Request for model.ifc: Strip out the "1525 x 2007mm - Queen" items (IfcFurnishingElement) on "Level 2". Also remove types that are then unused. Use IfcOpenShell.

First a look at what the model holds.

```python
import ifcopenshell
import ifcopenshell.util.element

model = ifcopenshell.open("model.ifc")
print(model.schema)
storey = next(s for s in model.by_type("IfcBuildingStorey") if s.Name == "Level 2")
furniture = [e for e in ifcopenshell.util.element.get_decomposition(storey) if e.is_a("IfcFurnishingElement")]
seen = {}
for e in furniture:
    element_type = ifcopenshell.util.element.get_type(e)
    name = element_type.Name if element_type not in (None, e) else None
    seen[name] = seen.get(name, 0) + 1
for name, count in sorted(seen.items(), key=str):
    print(count, "x", name)
```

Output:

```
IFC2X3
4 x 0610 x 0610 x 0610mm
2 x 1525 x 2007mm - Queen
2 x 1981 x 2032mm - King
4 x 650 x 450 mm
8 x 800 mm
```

```python
import ifcopenshell
import ifcopenshell.api.root
import ifcopenshell.util.element

model = ifcopenshell.open("model.ifc")

storey = next(s for s in model.by_type("IfcBuildingStorey") if s.Name == "Level 2")
furniture = [e for e in ifcopenshell.util.element.get_decomposition(storey) if e.is_a("IfcFurnishingElement")]
targets = [e for e in furniture if (t := ifcopenshell.util.element.get_type(e)) not in (None, e) and t.Name == "1525 x 2007mm - Queen"]
types = {ifcopenshell.util.element.get_type(e) for e in targets} - {None, *targets}

for e in targets:
    ifcopenshell.api.root.remove_product(model, product=e)
print(len(targets), "removed")

unused = [t for t in types if not ifcopenshell.util.element.get_types(t)]
for t in unused:
    ifcopenshell.api.root.remove_product(model, product=t)
print(len(unused), "unused types removed")

model.write("model_edited.ifc")
```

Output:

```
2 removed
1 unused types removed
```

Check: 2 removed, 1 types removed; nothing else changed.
